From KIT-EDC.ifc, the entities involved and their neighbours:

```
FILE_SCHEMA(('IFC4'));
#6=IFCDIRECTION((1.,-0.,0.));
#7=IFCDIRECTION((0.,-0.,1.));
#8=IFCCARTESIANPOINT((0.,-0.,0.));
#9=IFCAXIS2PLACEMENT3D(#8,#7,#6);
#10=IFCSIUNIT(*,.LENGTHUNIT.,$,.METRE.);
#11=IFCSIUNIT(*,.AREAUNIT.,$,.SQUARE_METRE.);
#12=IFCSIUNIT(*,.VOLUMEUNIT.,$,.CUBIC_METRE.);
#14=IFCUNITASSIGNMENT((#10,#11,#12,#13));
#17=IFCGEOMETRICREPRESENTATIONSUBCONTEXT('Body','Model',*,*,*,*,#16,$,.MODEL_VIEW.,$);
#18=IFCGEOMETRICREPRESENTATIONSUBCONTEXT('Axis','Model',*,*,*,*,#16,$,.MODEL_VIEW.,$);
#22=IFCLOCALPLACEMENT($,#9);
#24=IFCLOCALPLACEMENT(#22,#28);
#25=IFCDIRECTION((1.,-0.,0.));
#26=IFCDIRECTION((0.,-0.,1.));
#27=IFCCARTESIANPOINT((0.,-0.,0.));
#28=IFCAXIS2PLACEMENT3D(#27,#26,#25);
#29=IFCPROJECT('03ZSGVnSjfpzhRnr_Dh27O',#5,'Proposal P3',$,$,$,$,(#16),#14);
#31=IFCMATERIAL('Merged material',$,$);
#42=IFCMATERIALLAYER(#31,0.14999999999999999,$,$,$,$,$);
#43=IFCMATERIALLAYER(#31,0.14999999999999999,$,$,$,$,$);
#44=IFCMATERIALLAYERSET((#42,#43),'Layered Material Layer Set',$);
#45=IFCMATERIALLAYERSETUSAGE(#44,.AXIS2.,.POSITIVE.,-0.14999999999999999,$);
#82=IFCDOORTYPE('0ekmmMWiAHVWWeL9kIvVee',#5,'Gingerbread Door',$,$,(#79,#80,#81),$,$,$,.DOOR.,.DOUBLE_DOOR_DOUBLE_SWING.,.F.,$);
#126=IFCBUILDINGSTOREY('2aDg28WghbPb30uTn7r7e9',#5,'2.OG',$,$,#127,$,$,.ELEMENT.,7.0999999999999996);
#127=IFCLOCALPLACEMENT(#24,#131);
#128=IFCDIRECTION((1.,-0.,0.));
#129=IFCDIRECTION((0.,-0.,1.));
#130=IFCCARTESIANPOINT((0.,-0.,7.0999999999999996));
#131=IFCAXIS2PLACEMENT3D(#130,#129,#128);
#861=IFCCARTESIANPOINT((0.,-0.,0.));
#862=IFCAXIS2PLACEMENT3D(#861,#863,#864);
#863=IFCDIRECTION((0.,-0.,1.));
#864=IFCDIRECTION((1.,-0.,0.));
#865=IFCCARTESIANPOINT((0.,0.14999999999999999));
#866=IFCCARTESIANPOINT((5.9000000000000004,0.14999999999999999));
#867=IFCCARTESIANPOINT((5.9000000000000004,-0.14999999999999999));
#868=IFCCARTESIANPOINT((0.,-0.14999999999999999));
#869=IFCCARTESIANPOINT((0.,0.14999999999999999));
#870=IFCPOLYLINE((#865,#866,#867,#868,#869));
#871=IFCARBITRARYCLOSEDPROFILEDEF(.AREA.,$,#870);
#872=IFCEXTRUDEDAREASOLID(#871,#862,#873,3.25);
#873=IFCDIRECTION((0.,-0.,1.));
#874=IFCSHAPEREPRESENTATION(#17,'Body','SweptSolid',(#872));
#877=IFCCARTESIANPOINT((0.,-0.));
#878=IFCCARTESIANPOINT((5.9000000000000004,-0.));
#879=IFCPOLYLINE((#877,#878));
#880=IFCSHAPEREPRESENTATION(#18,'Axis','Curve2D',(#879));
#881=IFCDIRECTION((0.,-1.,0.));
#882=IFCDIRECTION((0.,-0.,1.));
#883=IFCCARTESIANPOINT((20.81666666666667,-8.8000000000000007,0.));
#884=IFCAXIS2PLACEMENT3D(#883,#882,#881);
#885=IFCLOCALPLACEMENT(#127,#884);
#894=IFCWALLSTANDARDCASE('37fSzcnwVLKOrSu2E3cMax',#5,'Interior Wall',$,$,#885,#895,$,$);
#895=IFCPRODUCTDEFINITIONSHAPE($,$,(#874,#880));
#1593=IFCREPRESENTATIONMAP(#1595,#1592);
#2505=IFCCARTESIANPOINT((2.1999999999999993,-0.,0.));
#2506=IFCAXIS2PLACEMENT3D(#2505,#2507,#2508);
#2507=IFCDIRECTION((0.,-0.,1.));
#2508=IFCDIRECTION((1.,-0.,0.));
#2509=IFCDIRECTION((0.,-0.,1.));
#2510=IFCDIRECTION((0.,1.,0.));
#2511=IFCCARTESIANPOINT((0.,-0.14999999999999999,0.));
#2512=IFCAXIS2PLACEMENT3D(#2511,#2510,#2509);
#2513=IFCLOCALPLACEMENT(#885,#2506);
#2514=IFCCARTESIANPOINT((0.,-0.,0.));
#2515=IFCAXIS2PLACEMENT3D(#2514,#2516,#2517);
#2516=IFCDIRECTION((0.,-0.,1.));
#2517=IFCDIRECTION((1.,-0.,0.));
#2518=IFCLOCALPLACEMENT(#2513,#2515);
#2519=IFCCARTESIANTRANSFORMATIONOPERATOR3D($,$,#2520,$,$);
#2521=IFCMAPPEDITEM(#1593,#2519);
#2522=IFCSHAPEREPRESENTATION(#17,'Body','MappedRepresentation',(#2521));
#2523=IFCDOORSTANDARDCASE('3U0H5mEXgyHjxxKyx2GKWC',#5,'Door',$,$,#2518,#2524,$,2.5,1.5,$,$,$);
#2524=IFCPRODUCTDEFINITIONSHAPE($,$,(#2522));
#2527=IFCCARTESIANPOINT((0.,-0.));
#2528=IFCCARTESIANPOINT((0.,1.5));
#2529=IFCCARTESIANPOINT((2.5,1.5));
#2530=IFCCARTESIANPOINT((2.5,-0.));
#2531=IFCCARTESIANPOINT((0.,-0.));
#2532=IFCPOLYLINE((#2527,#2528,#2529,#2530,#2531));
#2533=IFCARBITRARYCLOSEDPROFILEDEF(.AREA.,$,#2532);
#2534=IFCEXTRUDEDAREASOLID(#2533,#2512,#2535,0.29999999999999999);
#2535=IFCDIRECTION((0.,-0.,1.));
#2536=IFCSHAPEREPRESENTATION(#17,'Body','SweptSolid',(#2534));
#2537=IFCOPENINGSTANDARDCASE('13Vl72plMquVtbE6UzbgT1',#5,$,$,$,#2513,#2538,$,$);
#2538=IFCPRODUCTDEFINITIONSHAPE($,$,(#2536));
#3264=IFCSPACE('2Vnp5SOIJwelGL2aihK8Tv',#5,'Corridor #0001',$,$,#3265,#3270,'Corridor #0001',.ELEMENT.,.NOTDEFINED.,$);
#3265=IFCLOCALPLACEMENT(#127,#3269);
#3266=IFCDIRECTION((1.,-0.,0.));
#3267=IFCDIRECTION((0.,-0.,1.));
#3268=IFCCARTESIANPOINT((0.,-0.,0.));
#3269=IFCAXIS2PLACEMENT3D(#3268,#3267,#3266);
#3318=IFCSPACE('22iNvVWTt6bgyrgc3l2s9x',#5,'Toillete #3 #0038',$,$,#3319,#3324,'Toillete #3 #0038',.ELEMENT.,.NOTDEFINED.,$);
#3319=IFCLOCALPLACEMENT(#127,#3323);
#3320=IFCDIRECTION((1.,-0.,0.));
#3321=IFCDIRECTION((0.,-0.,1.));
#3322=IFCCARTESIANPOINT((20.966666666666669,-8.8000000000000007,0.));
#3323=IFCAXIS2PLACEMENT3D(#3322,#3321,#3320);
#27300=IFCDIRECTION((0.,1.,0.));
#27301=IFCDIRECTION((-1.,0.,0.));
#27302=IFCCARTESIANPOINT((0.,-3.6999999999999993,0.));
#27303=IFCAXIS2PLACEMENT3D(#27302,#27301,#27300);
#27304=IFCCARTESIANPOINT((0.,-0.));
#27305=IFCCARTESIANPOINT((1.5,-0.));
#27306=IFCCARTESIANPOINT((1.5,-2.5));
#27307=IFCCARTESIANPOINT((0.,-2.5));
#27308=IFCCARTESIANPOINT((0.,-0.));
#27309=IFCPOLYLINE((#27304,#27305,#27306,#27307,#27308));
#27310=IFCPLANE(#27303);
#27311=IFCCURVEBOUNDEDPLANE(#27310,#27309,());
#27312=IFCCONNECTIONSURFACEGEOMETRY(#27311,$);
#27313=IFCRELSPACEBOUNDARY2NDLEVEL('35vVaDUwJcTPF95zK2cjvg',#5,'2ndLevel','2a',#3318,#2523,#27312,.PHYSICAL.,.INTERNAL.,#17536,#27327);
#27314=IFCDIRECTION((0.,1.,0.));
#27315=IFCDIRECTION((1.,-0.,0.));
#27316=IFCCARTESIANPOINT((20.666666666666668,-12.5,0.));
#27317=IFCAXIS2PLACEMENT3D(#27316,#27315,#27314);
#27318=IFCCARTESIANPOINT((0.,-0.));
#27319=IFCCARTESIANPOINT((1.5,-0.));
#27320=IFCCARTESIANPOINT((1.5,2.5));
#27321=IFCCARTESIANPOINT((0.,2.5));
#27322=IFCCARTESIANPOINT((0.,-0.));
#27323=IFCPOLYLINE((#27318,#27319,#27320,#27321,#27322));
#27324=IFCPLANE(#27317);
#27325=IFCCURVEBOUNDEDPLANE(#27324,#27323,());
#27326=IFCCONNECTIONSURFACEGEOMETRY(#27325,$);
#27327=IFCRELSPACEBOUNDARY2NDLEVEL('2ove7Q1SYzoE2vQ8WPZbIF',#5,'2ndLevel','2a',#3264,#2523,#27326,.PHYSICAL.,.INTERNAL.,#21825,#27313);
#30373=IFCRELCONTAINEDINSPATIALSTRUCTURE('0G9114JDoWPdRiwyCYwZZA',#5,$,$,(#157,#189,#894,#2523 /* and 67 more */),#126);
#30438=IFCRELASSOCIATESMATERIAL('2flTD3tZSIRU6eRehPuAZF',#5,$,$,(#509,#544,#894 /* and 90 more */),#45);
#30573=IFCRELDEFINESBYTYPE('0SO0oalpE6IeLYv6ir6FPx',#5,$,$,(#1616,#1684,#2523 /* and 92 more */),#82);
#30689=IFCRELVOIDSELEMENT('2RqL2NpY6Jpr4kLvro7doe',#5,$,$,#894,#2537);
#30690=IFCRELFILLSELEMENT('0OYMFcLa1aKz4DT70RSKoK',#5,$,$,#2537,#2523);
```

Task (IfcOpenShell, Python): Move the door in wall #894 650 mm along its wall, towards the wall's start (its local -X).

```python
import numpy as np
import ifcopenshell
import ifcopenshell.api.geometry
import ifcopenshell.util.placement

model = ifcopenshell.open("KIT-EDC.ifc")

door = model.by_guid("3U0H5mEXgyHjxxKyx2GKWC")
opening = door.FillsVoids[0].RelatingOpeningElement
wall = opening.VoidsElements[0].RelatingBuildingElement

wall_matrix = ifcopenshell.util.placement.get_local_placement(wall.ObjectPlacement)
shift = wall_matrix[:3, 0] * -0.65
before = ifcopenshell.util.placement.get_local_placement(door.ObjectPlacement)[:3, 3].copy()

# The door is placed relative to its opening, so it follows when the opening moves.
matrix = ifcopenshell.util.placement.get_local_placement(opening.ObjectPlacement)
matrix[:3, 3] += shift
ifcopenshell.api.geometry.edit_object_placement(
    model, product=opening, matrix=matrix, is_si=False, should_transform_children=True
)

# Space boundary surfaces are stored in each space's coordinates; move them too.
for rel in door.ProvidesBoundaries:
    if not rel.ConnectionGeometry:
        continue
    surface = rel.ConnectionGeometry.SurfaceOnRelatingElement.BasisSurface
    space_matrix = ifcopenshell.util.placement.get_local_placement(rel.RelatingSpace.ObjectPlacement)
    point = np.array(surface.Position.Location.Coordinates) + space_matrix[:3, :3].T @ shift
    surface.Position = model.createIfcAxis2Placement3D(
        model.createIfcCartesianPoint(point.tolist()), surface.Position.Axis, surface.Position.RefDirection
    )

after = ifcopenshell.util.placement.get_local_placement(door.ObjectPlacement)[:3, 3]
print("door moved by", (after - before).round(3) + 0.0)

model.write("KIT-EDC_updated.ifc")
```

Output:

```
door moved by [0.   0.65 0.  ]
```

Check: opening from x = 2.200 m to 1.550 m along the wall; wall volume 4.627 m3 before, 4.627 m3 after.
